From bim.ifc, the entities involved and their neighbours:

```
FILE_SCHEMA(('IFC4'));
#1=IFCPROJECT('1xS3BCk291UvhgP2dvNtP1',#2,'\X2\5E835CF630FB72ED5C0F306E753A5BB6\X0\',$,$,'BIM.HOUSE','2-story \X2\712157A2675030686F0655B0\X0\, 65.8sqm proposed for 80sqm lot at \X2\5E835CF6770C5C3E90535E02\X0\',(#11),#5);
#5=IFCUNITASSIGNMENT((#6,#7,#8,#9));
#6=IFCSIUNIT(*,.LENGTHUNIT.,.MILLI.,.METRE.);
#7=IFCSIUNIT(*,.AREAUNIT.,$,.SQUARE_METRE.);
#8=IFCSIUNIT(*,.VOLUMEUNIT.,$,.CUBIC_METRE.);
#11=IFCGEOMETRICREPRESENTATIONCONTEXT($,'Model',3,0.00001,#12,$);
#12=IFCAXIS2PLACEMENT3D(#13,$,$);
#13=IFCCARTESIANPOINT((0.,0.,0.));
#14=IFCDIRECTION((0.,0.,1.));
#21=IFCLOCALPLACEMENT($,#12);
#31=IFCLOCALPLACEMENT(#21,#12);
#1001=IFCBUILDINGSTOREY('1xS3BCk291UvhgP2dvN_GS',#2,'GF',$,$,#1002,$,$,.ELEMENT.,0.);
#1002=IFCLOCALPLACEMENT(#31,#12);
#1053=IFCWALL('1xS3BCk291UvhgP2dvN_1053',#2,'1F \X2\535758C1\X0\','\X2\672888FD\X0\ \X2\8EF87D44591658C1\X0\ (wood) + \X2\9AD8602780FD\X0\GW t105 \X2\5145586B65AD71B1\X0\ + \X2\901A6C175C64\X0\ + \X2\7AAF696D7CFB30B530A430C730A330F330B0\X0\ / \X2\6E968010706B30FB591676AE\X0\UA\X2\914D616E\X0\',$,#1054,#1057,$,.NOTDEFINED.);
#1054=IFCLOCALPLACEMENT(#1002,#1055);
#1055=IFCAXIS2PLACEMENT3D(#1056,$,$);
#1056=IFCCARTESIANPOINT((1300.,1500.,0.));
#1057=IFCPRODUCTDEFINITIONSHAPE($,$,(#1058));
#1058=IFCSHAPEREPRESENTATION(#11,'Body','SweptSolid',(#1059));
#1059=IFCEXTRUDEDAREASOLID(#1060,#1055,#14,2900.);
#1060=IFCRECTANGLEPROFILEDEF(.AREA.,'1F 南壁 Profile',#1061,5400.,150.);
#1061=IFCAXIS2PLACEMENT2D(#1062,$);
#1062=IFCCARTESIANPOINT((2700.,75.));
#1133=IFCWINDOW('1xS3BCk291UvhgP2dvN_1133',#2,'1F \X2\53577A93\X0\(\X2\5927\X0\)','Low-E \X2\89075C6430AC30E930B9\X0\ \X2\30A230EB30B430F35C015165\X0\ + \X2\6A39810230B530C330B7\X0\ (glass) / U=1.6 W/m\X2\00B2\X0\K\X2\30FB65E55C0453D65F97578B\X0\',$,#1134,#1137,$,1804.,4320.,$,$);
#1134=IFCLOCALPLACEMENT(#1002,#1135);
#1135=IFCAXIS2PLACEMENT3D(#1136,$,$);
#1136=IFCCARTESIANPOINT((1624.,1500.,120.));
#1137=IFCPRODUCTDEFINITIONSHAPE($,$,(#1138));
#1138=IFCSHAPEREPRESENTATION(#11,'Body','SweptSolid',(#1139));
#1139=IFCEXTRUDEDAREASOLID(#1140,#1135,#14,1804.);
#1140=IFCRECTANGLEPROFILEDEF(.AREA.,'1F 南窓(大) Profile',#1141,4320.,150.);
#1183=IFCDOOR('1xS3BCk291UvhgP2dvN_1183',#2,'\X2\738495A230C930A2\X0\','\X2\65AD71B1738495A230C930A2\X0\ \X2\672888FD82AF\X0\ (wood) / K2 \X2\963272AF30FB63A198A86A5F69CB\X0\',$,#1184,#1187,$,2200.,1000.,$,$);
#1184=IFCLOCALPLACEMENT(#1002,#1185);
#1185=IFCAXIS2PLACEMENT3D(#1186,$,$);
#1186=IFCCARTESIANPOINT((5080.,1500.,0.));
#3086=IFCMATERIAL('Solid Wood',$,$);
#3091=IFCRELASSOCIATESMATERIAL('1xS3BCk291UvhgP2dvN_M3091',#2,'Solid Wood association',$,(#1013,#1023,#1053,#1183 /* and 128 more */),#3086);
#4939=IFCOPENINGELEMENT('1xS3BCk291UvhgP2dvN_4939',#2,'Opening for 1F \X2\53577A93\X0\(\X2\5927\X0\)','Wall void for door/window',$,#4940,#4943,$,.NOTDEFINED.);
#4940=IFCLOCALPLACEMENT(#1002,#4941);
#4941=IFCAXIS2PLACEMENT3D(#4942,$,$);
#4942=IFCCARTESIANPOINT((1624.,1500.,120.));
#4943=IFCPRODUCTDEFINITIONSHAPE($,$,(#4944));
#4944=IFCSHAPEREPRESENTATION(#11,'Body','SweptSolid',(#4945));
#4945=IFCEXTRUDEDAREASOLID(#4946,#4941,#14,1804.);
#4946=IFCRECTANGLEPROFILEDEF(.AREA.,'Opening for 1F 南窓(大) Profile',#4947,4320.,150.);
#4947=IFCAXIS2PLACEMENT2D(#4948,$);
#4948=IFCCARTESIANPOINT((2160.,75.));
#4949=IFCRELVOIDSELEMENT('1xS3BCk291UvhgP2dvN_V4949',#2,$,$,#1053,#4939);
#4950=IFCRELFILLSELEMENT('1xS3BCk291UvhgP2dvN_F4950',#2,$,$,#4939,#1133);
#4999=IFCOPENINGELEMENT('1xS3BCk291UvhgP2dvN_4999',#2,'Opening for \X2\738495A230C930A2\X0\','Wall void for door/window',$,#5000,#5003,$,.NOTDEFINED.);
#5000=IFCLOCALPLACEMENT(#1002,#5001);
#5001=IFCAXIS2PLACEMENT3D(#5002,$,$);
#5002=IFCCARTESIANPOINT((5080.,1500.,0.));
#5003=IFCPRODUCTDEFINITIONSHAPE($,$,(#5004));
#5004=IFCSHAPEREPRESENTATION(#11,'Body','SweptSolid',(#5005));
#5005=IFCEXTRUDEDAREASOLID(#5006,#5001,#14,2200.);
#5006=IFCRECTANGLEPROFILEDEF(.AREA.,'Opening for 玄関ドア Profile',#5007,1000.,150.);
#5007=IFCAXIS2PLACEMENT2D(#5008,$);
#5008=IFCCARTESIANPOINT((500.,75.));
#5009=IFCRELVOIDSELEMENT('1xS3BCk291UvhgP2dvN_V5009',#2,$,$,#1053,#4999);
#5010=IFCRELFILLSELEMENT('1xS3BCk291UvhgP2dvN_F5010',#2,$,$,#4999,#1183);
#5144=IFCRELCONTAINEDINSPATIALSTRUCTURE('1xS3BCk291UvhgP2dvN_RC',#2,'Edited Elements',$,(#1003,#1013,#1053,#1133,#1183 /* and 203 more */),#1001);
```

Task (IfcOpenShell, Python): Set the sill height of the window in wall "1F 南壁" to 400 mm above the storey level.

```python
import numpy as np
import ifcopenshell
import ifcopenshell.api.geometry
import ifcopenshell.geom
import ifcopenshell.util.element
import ifcopenshell.util.placement
import ifcopenshell.util.shape
import ifcopenshell.util.unit

model = ifcopenshell.open("bim.ifc")
unit_scale = ifcopenshell.util.unit.calculate_unit_scale(model)

window = model.by_id(1133)
opening = window.FillsVoids[0].RelatingOpeningElement
storey = ifcopenshell.util.element.get_container(window, ifc_class="IfcBuildingStorey")
level = ifcopenshell.util.placement.get_local_placement(storey.ObjectPlacement)[2, 3]

# The opening's origin need not be at the sill, so measure its lowest point.
shape = ifcopenshell.geom.create_shape(ifcopenshell.geom.settings(), opening)
bottom = ifcopenshell.util.shape.get_shape_bottom_elevation(shape, shape.geometry) / unit_scale
dz = level + 400.0 - bottom

shift = np.array([0.0, 0.0, dz])
# The window is not placed relative to its opening, so move both.
for product in (opening, window):
    matrix = ifcopenshell.util.placement.get_local_placement(product.ObjectPlacement)
    matrix[:3, 3] += shift
    ifcopenshell.api.geometry.edit_object_placement(model, product=product, matrix=matrix, is_si=False)

print(f"moved by {dz * unit_scale:+.3f} m")

model.write("bim_updated.ifc")
```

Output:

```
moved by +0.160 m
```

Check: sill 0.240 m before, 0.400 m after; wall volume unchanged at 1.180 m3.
